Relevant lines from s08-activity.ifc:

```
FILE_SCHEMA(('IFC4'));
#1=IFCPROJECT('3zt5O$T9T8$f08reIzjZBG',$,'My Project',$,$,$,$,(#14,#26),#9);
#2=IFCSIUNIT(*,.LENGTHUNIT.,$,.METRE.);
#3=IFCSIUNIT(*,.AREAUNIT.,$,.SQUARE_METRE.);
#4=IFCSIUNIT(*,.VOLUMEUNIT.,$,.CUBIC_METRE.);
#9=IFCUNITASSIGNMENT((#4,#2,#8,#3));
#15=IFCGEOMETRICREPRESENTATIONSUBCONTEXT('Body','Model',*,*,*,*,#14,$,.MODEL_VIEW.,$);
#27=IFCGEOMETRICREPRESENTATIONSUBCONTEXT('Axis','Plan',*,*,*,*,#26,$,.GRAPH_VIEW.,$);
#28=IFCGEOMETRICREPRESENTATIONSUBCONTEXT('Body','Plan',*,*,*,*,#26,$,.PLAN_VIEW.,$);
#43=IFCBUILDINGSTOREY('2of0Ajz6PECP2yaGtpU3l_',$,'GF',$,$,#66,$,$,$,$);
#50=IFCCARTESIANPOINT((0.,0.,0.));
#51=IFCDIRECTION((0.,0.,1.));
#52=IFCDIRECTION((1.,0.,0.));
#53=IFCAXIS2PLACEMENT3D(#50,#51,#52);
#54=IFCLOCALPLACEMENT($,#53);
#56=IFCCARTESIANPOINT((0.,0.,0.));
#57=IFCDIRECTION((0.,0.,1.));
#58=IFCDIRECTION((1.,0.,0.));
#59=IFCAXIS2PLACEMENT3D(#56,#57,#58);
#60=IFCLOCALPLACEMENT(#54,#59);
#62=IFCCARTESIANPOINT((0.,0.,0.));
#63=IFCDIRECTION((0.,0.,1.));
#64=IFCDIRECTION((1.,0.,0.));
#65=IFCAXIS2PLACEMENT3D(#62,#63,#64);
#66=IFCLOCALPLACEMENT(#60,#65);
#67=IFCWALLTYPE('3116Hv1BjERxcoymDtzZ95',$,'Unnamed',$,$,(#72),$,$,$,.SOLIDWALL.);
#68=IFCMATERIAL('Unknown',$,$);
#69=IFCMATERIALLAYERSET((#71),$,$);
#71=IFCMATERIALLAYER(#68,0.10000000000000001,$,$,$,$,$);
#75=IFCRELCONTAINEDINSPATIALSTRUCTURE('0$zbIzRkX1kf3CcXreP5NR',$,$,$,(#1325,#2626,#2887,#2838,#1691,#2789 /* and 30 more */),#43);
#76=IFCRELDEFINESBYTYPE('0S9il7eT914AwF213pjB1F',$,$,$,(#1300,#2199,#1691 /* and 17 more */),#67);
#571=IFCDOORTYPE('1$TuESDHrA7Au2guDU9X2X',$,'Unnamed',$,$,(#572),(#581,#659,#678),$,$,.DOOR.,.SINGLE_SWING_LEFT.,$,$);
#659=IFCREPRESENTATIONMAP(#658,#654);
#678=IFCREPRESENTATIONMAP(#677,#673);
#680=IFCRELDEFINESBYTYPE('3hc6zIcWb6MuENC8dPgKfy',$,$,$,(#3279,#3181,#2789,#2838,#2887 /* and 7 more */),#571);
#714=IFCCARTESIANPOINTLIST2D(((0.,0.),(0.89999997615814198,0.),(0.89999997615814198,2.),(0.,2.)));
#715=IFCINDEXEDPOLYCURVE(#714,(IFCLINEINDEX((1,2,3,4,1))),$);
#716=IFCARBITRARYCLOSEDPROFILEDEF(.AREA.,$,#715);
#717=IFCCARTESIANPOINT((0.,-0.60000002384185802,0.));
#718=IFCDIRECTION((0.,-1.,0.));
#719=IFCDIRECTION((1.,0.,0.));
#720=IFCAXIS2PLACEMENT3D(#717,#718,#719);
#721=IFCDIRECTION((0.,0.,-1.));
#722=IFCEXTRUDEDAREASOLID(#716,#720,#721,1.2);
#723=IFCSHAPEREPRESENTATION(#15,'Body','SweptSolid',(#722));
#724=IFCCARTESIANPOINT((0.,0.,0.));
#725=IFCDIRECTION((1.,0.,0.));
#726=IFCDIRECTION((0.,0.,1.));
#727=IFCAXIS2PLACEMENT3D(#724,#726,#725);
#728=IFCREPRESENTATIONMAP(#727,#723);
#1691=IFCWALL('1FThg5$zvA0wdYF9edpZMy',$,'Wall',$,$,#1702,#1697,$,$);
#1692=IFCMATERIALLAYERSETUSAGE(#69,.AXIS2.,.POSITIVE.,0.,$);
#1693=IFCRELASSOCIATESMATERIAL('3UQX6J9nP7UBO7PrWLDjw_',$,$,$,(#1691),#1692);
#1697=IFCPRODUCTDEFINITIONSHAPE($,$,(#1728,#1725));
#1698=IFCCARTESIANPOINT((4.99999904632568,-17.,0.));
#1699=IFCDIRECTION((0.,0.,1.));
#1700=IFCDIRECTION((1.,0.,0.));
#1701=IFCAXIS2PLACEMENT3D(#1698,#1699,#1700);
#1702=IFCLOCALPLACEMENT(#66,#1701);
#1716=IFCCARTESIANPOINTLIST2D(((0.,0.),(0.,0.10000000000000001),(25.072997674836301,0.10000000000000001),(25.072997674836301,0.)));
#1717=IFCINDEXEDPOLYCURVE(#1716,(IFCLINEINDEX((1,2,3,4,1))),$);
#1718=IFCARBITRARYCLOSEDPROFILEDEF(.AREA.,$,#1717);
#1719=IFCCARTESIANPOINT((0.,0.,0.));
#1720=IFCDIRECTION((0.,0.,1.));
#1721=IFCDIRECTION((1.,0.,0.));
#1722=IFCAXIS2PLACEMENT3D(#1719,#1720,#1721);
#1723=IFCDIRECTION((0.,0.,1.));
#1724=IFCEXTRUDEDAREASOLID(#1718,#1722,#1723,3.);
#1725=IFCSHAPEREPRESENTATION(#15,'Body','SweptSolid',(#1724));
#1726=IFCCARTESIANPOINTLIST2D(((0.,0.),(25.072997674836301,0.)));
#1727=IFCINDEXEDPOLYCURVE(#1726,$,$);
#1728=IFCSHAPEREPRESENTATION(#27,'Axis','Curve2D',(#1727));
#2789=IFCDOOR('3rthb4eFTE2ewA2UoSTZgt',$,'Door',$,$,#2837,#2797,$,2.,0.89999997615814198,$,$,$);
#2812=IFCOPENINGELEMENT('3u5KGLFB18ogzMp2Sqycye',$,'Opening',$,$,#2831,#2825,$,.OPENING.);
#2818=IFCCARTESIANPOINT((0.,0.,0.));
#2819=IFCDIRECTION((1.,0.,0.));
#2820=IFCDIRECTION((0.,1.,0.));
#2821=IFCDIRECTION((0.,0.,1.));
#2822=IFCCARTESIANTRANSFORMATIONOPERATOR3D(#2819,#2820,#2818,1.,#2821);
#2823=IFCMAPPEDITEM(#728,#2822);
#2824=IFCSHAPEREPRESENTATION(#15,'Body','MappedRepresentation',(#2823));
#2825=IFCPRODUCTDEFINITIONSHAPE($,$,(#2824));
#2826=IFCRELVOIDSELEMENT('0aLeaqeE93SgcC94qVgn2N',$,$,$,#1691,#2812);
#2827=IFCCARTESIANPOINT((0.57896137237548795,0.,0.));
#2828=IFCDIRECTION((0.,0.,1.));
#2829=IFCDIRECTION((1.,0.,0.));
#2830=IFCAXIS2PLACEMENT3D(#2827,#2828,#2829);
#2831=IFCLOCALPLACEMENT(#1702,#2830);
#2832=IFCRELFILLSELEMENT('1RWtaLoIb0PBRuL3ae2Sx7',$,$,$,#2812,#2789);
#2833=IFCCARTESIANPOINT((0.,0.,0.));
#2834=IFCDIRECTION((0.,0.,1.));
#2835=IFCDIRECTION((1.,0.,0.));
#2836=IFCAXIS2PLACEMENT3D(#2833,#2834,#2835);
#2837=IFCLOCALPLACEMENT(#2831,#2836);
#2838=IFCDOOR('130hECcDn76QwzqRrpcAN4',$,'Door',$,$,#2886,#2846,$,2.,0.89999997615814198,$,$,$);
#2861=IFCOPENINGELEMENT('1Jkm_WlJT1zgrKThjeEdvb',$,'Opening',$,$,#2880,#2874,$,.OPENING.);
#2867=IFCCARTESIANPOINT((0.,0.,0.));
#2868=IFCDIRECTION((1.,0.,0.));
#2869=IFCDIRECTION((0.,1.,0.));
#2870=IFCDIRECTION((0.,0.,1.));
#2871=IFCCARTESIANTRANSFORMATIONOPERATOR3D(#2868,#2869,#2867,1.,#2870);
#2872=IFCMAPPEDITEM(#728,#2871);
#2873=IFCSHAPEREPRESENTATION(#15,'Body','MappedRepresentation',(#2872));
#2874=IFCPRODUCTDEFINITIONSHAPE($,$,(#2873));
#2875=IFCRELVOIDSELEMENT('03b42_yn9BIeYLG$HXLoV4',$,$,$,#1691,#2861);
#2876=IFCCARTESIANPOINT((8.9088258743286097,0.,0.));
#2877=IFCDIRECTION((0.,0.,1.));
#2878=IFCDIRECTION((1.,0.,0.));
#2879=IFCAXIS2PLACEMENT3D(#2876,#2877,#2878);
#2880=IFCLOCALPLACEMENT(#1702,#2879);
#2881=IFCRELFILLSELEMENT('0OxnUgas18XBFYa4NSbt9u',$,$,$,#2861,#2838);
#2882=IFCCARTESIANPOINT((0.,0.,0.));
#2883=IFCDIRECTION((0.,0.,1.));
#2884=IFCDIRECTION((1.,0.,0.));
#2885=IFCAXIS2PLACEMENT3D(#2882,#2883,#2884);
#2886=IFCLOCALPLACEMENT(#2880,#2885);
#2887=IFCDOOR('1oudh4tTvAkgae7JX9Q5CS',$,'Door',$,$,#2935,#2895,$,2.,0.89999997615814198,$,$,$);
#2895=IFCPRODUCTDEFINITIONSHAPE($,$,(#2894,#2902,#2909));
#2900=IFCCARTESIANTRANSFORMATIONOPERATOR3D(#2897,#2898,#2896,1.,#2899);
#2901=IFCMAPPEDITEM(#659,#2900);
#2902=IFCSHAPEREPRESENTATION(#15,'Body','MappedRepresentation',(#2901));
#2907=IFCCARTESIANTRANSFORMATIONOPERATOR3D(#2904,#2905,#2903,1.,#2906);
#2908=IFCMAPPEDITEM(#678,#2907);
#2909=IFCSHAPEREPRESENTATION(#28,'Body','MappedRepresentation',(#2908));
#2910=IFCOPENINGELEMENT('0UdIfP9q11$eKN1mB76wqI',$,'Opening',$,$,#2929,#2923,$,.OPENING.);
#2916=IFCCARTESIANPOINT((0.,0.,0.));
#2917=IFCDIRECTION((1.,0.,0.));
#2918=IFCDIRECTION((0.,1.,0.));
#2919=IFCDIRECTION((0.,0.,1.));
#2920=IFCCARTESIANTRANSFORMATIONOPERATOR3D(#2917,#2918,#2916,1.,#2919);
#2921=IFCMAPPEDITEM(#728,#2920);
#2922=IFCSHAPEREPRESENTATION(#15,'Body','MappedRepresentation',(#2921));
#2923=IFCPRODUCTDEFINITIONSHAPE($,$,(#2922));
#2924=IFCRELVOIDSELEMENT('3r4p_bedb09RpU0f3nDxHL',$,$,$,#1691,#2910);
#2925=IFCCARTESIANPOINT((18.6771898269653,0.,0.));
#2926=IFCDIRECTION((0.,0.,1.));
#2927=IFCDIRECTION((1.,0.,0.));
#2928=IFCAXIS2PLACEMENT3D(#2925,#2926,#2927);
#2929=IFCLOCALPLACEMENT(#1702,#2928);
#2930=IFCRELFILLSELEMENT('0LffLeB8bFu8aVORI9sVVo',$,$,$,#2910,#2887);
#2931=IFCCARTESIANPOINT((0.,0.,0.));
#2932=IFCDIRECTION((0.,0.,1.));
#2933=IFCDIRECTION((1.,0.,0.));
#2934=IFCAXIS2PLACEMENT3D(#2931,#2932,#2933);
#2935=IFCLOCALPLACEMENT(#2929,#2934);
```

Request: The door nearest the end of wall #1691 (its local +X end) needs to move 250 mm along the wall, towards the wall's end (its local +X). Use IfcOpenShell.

```python
import ifcopenshell
import ifcopenshell.api.geometry
import ifcopenshell.util.placement

model = ifcopenshell.open("s08-activity.ifc")

door = model.by_guid("1oudh4tTvAkgae7JX9Q5CS")
opening = door.FillsVoids[0].RelatingOpeningElement
wall = opening.VoidsElements[0].RelatingBuildingElement

wall_matrix = ifcopenshell.util.placement.get_local_placement(wall.ObjectPlacement)
shift = wall_matrix[:3, 0] * 0.25
before = ifcopenshell.util.placement.get_local_placement(door.ObjectPlacement)[:3, 3].copy()

# The door is placed relative to its opening, so it follows when the opening moves.
matrix = ifcopenshell.util.placement.get_local_placement(opening.ObjectPlacement)
matrix[:3, 3] += shift
ifcopenshell.api.geometry.edit_object_placement(
    model, product=opening, matrix=matrix, is_si=False, should_transform_children=True
)

after = ifcopenshell.util.placement.get_local_placement(door.ObjectPlacement)[:3, 3]
print("door moved by", (after - before).round(3) + 0.0)

model.write("s08-activity_rev.ifc")
```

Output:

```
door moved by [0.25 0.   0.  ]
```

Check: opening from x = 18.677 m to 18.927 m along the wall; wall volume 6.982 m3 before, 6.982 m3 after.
